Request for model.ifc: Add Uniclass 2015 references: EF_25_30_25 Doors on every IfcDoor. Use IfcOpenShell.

First a look at what the model holds.

```python
import ifcopenshell

model = ifcopenshell.open("model.ifc")
print(model.schema)
print("classifications:", [c.Name for c in model.by_type("IfcClassification")])
for ifc_class in ("IfcDoor", "IfcRoof", "IfcStair", "IfcWall", "IfcWindow"):
    print(ifc_class, len(model.by_type(ifc_class)))
```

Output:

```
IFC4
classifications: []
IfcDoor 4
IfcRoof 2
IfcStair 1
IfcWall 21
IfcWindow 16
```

```python
import ifcopenshell
import ifcopenshell.api.classification

model = ifcopenshell.open("model.ifc")

system = ifcopenshell.api.classification.add_classification(model, classification="Uniclass 2015")

codes = {
    "IfcDoor": ("EF_25_30_25", "Doors"),
}
for ifc_class, (code, name) in codes.items():
    products = model.by_type(ifc_class)
    ifcopenshell.api.classification.add_reference(
        model, products=products, classification=system, identification=code, name=name
    )
    print(code, len(products))

model.write("model_v2.ifc")
```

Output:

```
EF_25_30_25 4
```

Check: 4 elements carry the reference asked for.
